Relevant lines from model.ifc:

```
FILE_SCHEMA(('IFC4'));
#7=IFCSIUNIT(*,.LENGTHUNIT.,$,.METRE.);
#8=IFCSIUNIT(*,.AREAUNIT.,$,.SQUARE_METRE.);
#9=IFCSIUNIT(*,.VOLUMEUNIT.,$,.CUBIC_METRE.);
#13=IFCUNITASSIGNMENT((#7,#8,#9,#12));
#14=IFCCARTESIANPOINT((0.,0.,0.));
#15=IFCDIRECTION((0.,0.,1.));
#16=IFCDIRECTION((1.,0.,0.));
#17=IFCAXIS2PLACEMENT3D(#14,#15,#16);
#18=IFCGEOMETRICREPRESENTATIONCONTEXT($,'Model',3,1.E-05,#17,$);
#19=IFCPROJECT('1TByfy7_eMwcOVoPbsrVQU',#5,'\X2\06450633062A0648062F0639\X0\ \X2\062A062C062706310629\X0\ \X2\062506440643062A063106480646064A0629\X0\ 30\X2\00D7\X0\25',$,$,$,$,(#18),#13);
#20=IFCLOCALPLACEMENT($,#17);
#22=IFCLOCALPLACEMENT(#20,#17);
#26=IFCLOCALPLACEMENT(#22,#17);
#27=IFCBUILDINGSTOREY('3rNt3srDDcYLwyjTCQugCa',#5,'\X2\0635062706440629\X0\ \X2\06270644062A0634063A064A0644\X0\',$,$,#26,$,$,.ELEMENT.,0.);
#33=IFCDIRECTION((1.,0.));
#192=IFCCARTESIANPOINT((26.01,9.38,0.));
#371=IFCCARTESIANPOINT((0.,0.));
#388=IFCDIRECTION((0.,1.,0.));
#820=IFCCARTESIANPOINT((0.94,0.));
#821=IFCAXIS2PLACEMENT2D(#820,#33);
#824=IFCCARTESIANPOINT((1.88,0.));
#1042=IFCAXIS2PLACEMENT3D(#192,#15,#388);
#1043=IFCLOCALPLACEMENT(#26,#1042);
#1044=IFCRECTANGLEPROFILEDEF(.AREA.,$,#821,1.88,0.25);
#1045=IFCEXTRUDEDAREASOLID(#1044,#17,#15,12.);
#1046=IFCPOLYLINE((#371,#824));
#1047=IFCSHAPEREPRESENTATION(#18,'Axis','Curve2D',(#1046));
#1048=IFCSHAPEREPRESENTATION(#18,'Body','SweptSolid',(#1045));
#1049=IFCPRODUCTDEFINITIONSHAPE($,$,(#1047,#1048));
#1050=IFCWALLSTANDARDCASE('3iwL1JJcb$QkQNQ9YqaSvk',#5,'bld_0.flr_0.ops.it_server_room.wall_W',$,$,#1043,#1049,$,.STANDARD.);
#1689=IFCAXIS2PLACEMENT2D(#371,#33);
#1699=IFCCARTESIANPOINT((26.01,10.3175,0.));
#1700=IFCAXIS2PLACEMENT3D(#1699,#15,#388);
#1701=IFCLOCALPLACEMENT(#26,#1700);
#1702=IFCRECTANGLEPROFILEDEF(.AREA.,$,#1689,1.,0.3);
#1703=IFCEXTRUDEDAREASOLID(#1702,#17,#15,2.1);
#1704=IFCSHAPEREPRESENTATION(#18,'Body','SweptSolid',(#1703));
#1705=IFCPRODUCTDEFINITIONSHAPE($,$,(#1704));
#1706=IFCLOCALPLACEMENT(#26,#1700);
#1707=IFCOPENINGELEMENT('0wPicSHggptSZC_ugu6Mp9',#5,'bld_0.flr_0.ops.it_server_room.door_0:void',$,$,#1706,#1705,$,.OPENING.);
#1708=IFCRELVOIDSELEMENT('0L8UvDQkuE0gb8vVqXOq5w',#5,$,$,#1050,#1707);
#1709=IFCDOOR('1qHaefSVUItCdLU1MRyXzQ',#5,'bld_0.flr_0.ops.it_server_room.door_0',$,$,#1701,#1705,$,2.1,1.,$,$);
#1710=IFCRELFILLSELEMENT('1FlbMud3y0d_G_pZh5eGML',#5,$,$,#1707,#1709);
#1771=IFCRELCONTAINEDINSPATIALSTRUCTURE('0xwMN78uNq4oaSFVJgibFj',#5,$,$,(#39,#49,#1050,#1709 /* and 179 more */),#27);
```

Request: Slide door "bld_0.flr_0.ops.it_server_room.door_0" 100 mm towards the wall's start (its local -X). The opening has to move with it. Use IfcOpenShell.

```python
import ifcopenshell
import ifcopenshell.api.geometry
import ifcopenshell.util.placement

model = ifcopenshell.open("model.ifc")

door = model.by_guid("1qHaefSVUItCdLU1MRyXzQ")
opening = door.FillsVoids[0].RelatingOpeningElement
wall = opening.VoidsElements[0].RelatingBuildingElement

wall_matrix = ifcopenshell.util.placement.get_local_placement(wall.ObjectPlacement)
shift = wall_matrix[:3, 0] * -0.1
before = ifcopenshell.util.placement.get_local_placement(door.ObjectPlacement)[:3, 3].copy()

# The door is not placed relative to its opening, so move both.
for product in (opening, door):
    matrix = ifcopenshell.util.placement.get_local_placement(product.ObjectPlacement)
    matrix[:3, 3] += shift
    ifcopenshell.api.geometry.edit_object_placement(model, product=product, matrix=matrix, is_si=False)

after = ifcopenshell.util.placement.get_local_placement(door.ObjectPlacement)[:3, 3]
print("door moved by", (after - before).round(3) + 0.0)

model.write("model_updated.ifc")
```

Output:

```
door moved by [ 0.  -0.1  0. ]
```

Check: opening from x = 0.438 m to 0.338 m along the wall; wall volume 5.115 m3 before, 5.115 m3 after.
